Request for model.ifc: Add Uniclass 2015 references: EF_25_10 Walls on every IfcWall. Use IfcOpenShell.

First a look at what the model holds.

```python
import ifcopenshell

model = ifcopenshell.open("model.ifc")
print(model.schema)
print("classifications:", [c.Name for c in model.by_type("IfcClassification")])
for ifc_class in ("IfcDoor", "IfcRoof", "IfcStair", "IfcWall", "IfcWindow"):
    print(ifc_class, len(model.by_type(ifc_class)))
```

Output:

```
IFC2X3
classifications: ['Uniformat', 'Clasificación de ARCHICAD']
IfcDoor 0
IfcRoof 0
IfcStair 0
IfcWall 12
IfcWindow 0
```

```python
import ifcopenshell
import ifcopenshell.api.classification

model = ifcopenshell.open("model.ifc")

# IFC2X3 requires Source and Edition and has no link from the project to the system.
system = model.create_entity("IfcClassification", Source="NBS", Edition="2015", Name="Uniclass 2015")

codes = {
    "IfcWall": ("EF_25_10", "Walls"),
}
for ifc_class, (code, name) in codes.items():
    products = model.by_type(ifc_class)
    ifcopenshell.api.classification.add_reference(
        model, products=products, classification=system, identification=code, name=name
    )
    print(code, len(products))

model.write("model_updated.ifc")
```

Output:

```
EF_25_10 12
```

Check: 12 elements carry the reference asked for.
